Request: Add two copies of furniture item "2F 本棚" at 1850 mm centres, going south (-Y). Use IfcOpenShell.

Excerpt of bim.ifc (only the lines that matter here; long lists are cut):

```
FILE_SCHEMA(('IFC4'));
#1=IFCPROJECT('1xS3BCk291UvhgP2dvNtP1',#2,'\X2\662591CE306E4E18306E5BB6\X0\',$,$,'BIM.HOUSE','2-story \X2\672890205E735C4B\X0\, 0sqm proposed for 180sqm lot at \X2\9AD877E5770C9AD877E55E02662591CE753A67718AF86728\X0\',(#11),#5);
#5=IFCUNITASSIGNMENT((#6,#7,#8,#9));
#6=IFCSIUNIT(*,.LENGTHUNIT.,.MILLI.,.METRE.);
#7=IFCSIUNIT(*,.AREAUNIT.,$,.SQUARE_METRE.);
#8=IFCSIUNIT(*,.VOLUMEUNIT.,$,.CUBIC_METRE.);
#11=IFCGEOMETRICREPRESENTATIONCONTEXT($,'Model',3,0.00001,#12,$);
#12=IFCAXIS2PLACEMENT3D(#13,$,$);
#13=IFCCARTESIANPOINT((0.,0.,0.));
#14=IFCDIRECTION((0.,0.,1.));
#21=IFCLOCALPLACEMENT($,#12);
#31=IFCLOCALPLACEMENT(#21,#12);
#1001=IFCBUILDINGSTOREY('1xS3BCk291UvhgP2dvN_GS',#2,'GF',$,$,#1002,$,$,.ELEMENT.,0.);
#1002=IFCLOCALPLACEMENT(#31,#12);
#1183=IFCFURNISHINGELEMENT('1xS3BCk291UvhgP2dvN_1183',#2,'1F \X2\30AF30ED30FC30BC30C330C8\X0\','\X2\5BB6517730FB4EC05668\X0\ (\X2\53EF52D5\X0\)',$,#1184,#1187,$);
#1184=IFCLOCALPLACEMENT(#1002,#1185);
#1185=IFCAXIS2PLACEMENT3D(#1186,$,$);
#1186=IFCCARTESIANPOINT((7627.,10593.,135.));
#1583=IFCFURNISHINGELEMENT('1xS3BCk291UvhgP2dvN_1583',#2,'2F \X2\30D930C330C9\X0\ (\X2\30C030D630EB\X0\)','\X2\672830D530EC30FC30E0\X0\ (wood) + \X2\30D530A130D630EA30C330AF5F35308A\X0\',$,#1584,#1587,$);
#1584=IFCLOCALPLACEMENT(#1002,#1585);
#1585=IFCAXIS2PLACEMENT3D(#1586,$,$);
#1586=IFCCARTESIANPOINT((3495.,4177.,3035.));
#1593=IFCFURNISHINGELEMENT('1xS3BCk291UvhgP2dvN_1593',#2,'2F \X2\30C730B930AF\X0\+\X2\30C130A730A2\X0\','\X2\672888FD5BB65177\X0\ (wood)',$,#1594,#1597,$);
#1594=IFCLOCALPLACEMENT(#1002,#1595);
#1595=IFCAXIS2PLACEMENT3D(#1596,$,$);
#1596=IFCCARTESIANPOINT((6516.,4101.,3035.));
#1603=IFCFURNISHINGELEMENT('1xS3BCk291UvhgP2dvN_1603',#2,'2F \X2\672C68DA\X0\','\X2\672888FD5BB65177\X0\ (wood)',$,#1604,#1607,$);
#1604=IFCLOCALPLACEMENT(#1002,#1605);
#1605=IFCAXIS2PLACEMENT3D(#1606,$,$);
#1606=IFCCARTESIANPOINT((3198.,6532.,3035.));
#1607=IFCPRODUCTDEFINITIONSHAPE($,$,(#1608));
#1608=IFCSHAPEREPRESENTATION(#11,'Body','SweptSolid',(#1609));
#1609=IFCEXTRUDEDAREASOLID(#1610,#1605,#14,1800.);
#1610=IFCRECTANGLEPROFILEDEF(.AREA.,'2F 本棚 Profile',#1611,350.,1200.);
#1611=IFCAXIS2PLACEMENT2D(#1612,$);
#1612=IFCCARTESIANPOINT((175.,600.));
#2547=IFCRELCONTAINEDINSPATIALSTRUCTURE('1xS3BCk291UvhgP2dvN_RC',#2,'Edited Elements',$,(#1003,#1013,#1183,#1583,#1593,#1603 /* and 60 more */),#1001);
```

```python
import numpy as np
import ifcopenshell
import ifcopenshell.api.geometry
import ifcopenshell.api.root
import ifcopenshell.util.element
import ifcopenshell.util.placement
import ifcopenshell.util.unit

model = ifcopenshell.open("bim.ifc")
unit_scale = ifcopenshell.util.unit.calculate_unit_scale(model)


def reuse_history(source, copy):
    """copy_class also copies each property set's owner history, people and application; keep the originals."""
    for rel in copy.IsDefinedBy:
        if rel.is_a("IfcRelDefinesByProperties") and (history := rel.RelatingPropertyDefinition.OwnerHistory):
            rel.RelatingPropertyDefinition.OwnerHistory = source.OwnerHistory
            ifcopenshell.util.element.remove_deep2(model, history)


source = model.by_guid("1xS3BCk291UvhgP2dvN_1603")
base = ifcopenshell.util.placement.get_local_placement(source.ObjectPlacement)
step = np.array([0.0, -1.0, 0.0]) * 1.85 / unit_scale

for i in range(1, 3):
    copy = ifcopenshell.api.root.copy_class(model, product=source)
    copy.Representation = ifcopenshell.util.element.copy_deep(
        model, source.Representation, exclude=["IfcGeometricRepresentationContext", "IfcRepresentationMap"]
    )
    reuse_history(source, copy)
    matrix = base.copy()
    matrix[:3, 3] += i * step
    print("added at", matrix[:3, 3].round(3) + 0.0)
    ifcopenshell.api.geometry.edit_object_placement(model, product=copy, matrix=matrix, is_si=False)

model.write("bim_updated.ifc")
```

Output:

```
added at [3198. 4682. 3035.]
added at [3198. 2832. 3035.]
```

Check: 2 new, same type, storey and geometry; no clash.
